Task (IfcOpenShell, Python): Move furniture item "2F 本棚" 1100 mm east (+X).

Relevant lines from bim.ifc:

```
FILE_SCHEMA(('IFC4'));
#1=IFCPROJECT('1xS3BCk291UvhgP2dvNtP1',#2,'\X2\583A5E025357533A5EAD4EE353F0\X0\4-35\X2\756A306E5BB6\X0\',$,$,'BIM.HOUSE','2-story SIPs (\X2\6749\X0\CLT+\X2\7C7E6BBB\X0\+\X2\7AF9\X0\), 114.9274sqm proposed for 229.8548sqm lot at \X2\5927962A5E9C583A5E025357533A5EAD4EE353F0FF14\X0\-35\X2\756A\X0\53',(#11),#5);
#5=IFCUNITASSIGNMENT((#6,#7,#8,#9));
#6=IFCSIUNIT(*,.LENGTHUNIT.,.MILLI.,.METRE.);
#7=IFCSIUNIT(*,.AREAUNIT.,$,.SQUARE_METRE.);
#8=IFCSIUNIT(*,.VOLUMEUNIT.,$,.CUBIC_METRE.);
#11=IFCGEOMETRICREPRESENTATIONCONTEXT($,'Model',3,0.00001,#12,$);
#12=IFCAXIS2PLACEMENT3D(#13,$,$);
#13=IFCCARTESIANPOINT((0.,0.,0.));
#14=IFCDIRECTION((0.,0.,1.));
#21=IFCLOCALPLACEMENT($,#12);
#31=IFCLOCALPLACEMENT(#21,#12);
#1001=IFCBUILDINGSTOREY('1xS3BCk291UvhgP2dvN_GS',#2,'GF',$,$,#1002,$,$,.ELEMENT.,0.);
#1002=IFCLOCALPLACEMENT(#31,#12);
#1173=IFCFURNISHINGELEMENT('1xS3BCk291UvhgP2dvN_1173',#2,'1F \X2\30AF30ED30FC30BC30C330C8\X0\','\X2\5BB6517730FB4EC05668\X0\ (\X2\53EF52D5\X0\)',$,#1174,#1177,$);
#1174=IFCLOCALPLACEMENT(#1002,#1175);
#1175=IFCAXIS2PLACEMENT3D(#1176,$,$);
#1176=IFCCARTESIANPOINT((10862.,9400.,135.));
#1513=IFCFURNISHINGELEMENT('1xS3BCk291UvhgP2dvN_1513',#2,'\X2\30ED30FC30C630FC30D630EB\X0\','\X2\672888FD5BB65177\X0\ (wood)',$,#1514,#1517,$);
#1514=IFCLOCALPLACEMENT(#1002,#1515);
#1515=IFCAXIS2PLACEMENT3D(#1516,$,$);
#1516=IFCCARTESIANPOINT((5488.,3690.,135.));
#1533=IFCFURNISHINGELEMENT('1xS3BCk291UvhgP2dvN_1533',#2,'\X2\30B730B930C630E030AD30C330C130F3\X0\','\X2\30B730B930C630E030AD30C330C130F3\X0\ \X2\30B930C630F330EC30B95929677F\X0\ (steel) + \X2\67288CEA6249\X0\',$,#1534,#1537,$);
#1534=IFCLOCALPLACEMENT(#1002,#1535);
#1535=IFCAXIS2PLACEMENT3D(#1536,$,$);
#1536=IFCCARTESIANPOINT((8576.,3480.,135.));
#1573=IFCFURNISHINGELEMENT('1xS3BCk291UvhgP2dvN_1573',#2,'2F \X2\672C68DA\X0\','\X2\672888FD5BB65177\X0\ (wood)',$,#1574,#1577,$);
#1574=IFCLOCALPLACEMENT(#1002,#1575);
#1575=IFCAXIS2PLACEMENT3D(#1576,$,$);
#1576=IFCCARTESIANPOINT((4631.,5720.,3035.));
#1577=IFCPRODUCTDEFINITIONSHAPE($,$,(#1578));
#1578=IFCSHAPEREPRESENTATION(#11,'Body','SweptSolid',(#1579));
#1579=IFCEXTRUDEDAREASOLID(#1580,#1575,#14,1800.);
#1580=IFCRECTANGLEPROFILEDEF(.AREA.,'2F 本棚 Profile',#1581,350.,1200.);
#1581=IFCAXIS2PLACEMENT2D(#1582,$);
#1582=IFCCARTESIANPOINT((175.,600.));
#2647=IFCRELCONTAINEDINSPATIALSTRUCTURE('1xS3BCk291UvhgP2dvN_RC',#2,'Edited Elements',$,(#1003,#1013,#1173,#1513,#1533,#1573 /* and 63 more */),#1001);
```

```python
import ifcopenshell
import ifcopenshell.api.geometry
import ifcopenshell.util.placement
import ifcopenshell.util.unit

model = ifcopenshell.open("bim.ifc")
unit_scale = ifcopenshell.util.unit.calculate_unit_scale(model)

item = model.by_guid("1xS3BCk291UvhgP2dvN_1573")
matrix = ifcopenshell.util.placement.get_local_placement(item.ObjectPlacement)
matrix[0, 3] += 1.1 / unit_scale
ifcopenshell.api.geometry.edit_object_placement(model, product=item, matrix=matrix, is_si=False)

print(ifcopenshell.util.placement.get_local_placement(item.ObjectPlacement).round(3) + 0.0)

model.write("bim-out.ifc")
```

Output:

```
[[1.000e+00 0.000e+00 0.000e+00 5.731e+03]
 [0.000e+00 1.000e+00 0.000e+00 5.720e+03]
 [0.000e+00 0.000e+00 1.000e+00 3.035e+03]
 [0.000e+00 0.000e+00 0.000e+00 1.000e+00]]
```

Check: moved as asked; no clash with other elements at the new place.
